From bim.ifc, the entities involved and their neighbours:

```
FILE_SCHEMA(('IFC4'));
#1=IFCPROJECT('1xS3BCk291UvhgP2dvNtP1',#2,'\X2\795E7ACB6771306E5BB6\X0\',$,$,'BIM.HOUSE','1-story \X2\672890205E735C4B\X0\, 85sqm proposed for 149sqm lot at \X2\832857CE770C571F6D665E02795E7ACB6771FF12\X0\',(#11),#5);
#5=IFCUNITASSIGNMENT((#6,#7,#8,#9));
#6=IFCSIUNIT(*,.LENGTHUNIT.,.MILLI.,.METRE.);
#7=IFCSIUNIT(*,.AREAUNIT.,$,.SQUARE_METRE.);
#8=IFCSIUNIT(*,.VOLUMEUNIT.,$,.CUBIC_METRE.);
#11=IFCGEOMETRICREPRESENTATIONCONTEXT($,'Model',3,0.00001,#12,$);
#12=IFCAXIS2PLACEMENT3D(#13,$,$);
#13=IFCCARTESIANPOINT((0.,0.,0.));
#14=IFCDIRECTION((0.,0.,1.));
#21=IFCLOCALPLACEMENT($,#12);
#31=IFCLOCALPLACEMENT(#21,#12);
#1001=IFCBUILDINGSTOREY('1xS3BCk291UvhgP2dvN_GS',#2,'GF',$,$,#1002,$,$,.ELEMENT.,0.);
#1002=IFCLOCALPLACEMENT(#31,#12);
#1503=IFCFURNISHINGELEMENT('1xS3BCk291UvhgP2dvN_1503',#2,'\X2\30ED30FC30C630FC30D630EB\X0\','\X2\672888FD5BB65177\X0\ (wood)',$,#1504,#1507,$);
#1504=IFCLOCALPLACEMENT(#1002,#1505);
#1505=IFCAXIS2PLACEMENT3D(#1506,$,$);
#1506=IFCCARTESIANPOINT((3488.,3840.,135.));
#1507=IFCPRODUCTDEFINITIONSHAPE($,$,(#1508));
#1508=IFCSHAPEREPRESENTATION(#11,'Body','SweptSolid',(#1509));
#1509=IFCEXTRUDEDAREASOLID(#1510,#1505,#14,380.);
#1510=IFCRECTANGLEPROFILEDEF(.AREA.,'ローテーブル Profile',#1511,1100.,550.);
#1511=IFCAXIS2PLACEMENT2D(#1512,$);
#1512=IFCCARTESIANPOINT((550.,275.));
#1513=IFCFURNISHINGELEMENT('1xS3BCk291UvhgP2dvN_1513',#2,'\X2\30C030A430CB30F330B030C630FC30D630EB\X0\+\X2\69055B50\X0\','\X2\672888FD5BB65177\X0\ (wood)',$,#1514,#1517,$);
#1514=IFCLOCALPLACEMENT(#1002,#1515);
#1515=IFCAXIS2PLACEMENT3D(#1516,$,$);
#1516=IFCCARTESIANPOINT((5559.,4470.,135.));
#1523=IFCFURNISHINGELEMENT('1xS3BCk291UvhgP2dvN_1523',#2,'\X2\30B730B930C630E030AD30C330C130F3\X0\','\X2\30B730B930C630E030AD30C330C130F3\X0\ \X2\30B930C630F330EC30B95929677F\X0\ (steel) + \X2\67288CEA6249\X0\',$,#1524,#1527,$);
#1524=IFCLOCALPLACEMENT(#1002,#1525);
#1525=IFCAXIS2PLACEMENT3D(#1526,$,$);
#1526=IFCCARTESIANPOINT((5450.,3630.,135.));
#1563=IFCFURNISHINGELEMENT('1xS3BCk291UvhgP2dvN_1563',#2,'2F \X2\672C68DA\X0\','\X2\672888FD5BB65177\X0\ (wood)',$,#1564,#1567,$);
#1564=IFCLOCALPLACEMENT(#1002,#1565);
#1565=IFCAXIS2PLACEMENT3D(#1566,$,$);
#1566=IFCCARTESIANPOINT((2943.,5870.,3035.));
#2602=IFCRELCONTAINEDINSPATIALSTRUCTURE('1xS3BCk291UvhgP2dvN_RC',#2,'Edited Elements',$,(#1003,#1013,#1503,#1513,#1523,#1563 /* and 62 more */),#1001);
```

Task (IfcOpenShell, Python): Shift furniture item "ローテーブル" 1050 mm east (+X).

```python
import ifcopenshell
import ifcopenshell.api.geometry
import ifcopenshell.util.placement
import ifcopenshell.util.unit

model = ifcopenshell.open("bim.ifc")
unit_scale = ifcopenshell.util.unit.calculate_unit_scale(model)

item = model.by_id(1503)
matrix = ifcopenshell.util.placement.get_local_placement(item.ObjectPlacement)
matrix[0, 3] += 1.05 / unit_scale
ifcopenshell.api.geometry.edit_object_placement(model, product=item, matrix=matrix, is_si=False)

print(ifcopenshell.util.placement.get_local_placement(item.ObjectPlacement).round(3) + 0.0)

model.write("bim-out.ifc")
```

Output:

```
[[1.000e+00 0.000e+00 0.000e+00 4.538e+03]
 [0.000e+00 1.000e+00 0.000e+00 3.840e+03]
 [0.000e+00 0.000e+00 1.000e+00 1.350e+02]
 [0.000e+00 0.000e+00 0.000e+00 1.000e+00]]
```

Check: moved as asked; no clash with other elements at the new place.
